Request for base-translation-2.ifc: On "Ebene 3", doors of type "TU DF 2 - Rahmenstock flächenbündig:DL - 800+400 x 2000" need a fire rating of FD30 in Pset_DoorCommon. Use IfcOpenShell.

First a look at what the model holds.

```python
import ifcopenshell
import ifcopenshell.util.element

model = ifcopenshell.open("base-translation-2.ifc")
print(model.schema)
storey = next(s for s in model.by_type("IfcBuildingStorey") if s.Name == "Ebene 3")
doors = [e for e in ifcopenshell.util.element.get_decomposition(storey) if e.is_a("IfcDoor")]
seen = {}
for e in doors:
    element_type = ifcopenshell.util.element.get_type(e)
    key = (element_type.Name if element_type != e and element_type else None, ifcopenshell.util.element.get_pset(e, "Pset_DoorCommon", "FireRating"))
    seen[key] = seen.get(key, 0) + 1
for (name, value), count in sorted(seen.items(), key=str):
    print(count, "x", name, "|", value)
```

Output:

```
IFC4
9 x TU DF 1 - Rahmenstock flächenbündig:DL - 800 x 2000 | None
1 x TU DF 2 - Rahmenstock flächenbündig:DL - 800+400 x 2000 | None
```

```python
import ifcopenshell
import ifcopenshell.api.pset
import ifcopenshell.util.element

model = ifcopenshell.open("base-translation-2.ifc")

storey = next(s for s in model.by_type("IfcBuildingStorey") if s.Name == "Ebene 3")
doors = [e for e in ifcopenshell.util.element.get_decomposition(storey) if e.is_a("IfcDoor")]

count = 0
for e in doors:
    element_type = ifcopenshell.util.element.get_type(e)
    if element_type in (None, e) or element_type.Name != "TU DF 2 - Rahmenstock flächenbündig:DL - 800+400 x 2000":
        continue
    # add_pset returns the element's existing set when there is one.
    pset = ifcopenshell.api.pset.add_pset(model, product=e, name="Pset_DoorCommon")
    ifcopenshell.api.pset.edit_pset(model, pset=pset, properties={"FireRating": "FD30"})
    count += 1

print(count, "doors updated")

model.write("base-translation-2_v2.ifc")
```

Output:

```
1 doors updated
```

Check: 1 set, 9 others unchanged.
